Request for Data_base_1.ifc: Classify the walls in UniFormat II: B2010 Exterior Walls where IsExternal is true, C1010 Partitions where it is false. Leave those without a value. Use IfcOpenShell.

First a look at what the model holds.

```python
import ifcopenshell
import ifcopenshell.util.element

model = ifcopenshell.open("Data_base_1.ifc")
print(model.schema)
print("classifications:", [c.Name for c in model.by_type("IfcClassification")])
values = [ifcopenshell.util.element.get_pset(e, "Pset_WallCommon", "IsExternal") for e in model.by_type("IfcWall")]
for value in (True, False, None):
    print("IsExternal", value, values.count(value))
```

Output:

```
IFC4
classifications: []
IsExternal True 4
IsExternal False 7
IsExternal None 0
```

```python
import ifcopenshell
import ifcopenshell.api.classification
import ifcopenshell.util.element

model = ifcopenshell.open("Data_base_1.ifc")

system = ifcopenshell.api.classification.add_classification(model, classification="UniFormat II")

walls = model.by_type("IfcWall")
external = {e: ifcopenshell.util.element.get_pset(e, "Pset_WallCommon", "IsExternal") for e in walls}
for flag, code, name in ((True, "B2010", "Exterior Walls"), (False, "C1010", "Partitions")):
    products = [e for e in walls if external[e] is flag]
    ifcopenshell.api.classification.add_reference(
        model, products=products, classification=system, identification=code, name=name
    )
    print(code, len(products))

model.write("Data_base_1-out.ifc")
```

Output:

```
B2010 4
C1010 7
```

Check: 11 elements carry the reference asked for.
